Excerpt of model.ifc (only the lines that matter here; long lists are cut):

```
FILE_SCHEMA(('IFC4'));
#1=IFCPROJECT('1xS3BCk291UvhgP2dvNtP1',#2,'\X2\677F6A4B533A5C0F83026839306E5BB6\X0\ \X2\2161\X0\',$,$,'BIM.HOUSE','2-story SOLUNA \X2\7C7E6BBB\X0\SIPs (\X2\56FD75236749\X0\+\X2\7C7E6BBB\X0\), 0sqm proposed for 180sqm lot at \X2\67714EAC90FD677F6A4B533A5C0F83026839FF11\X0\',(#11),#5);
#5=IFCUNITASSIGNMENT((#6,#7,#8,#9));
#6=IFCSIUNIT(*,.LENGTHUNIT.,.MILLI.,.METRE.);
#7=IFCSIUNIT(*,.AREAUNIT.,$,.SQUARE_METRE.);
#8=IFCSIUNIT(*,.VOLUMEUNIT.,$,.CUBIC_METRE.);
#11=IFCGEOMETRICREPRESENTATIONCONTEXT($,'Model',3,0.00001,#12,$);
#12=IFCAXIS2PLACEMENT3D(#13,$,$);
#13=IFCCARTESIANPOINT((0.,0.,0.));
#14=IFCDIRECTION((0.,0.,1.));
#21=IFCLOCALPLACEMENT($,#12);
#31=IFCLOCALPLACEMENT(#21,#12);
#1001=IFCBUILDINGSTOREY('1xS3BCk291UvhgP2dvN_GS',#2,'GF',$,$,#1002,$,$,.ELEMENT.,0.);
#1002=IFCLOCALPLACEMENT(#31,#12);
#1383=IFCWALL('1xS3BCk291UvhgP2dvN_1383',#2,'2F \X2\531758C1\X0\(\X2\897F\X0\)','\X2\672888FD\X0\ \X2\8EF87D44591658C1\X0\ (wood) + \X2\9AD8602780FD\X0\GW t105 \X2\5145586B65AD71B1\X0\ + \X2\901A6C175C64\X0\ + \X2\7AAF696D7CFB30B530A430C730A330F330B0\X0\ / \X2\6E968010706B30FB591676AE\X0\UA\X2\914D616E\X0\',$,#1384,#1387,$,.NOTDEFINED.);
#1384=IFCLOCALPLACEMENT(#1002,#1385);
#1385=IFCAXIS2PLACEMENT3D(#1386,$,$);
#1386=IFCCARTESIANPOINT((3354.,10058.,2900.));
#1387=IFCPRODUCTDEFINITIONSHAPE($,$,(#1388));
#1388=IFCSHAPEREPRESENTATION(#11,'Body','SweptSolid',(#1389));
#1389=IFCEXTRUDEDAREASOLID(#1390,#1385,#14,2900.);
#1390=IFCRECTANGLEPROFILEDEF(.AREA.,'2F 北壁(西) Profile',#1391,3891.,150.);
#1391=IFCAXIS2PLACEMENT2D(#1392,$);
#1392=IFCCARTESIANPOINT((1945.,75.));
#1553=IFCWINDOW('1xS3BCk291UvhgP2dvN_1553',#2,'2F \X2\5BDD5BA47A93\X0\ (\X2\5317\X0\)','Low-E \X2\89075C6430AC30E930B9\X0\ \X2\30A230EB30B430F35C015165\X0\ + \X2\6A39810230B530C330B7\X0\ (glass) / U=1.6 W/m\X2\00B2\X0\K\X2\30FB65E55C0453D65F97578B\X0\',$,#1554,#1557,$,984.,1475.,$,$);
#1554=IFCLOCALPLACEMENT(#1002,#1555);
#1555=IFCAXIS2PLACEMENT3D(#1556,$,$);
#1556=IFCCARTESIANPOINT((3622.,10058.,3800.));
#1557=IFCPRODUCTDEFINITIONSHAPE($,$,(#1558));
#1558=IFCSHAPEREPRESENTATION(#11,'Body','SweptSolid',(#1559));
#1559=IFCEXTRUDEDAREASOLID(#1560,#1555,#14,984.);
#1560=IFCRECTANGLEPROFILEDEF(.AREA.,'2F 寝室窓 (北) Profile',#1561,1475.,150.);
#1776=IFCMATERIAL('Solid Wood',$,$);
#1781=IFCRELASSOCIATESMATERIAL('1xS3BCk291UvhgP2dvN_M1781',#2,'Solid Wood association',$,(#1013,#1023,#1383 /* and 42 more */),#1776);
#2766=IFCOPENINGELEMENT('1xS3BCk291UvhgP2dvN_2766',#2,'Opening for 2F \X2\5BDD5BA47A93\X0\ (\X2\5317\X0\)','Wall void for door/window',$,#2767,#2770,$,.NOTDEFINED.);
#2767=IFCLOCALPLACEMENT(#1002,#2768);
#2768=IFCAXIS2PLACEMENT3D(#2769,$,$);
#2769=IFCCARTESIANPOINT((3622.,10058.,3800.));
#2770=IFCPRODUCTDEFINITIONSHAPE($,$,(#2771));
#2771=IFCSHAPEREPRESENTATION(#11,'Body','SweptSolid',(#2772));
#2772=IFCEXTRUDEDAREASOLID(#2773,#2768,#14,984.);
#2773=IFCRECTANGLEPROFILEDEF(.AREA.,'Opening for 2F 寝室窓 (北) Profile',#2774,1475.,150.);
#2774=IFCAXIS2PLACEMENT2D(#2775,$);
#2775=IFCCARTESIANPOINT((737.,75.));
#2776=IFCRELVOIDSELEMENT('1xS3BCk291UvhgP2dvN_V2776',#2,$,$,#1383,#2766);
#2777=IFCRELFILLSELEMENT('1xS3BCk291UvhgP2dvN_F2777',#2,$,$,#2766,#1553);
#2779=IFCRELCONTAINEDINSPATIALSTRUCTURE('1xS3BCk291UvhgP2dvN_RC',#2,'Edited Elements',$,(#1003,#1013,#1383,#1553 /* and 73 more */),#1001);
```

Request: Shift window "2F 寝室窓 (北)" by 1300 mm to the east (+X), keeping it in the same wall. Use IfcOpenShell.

```python
import ifcopenshell
import ifcopenshell.api.geometry
import ifcopenshell.util.placement

model = ifcopenshell.open("model.ifc")

window = model.by_guid("1xS3BCk291UvhgP2dvN_1553")
opening = window.FillsVoids[0].RelatingOpeningElement
wall = opening.VoidsElements[0].RelatingBuildingElement

wall_matrix = ifcopenshell.util.placement.get_local_placement(wall.ObjectPlacement)
shift = wall_matrix[:3, 0] * 1300.0
before = ifcopenshell.util.placement.get_local_placement(window.ObjectPlacement)[:3, 3].copy()

# The window is not placed relative to its opening, so move both.
for product in (opening, window):
    matrix = ifcopenshell.util.placement.get_local_placement(product.ObjectPlacement)
    matrix[:3, 3] += shift
    ifcopenshell.api.geometry.edit_object_placement(model, product=product, matrix=matrix, is_si=False)

after = ifcopenshell.util.placement.get_local_placement(window.ObjectPlacement)[:3, 3]
print("window moved by", (after - before).round(3) + 0.0)

model.write("model_v2.ifc")
```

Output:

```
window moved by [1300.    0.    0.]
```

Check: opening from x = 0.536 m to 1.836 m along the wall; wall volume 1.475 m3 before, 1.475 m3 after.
